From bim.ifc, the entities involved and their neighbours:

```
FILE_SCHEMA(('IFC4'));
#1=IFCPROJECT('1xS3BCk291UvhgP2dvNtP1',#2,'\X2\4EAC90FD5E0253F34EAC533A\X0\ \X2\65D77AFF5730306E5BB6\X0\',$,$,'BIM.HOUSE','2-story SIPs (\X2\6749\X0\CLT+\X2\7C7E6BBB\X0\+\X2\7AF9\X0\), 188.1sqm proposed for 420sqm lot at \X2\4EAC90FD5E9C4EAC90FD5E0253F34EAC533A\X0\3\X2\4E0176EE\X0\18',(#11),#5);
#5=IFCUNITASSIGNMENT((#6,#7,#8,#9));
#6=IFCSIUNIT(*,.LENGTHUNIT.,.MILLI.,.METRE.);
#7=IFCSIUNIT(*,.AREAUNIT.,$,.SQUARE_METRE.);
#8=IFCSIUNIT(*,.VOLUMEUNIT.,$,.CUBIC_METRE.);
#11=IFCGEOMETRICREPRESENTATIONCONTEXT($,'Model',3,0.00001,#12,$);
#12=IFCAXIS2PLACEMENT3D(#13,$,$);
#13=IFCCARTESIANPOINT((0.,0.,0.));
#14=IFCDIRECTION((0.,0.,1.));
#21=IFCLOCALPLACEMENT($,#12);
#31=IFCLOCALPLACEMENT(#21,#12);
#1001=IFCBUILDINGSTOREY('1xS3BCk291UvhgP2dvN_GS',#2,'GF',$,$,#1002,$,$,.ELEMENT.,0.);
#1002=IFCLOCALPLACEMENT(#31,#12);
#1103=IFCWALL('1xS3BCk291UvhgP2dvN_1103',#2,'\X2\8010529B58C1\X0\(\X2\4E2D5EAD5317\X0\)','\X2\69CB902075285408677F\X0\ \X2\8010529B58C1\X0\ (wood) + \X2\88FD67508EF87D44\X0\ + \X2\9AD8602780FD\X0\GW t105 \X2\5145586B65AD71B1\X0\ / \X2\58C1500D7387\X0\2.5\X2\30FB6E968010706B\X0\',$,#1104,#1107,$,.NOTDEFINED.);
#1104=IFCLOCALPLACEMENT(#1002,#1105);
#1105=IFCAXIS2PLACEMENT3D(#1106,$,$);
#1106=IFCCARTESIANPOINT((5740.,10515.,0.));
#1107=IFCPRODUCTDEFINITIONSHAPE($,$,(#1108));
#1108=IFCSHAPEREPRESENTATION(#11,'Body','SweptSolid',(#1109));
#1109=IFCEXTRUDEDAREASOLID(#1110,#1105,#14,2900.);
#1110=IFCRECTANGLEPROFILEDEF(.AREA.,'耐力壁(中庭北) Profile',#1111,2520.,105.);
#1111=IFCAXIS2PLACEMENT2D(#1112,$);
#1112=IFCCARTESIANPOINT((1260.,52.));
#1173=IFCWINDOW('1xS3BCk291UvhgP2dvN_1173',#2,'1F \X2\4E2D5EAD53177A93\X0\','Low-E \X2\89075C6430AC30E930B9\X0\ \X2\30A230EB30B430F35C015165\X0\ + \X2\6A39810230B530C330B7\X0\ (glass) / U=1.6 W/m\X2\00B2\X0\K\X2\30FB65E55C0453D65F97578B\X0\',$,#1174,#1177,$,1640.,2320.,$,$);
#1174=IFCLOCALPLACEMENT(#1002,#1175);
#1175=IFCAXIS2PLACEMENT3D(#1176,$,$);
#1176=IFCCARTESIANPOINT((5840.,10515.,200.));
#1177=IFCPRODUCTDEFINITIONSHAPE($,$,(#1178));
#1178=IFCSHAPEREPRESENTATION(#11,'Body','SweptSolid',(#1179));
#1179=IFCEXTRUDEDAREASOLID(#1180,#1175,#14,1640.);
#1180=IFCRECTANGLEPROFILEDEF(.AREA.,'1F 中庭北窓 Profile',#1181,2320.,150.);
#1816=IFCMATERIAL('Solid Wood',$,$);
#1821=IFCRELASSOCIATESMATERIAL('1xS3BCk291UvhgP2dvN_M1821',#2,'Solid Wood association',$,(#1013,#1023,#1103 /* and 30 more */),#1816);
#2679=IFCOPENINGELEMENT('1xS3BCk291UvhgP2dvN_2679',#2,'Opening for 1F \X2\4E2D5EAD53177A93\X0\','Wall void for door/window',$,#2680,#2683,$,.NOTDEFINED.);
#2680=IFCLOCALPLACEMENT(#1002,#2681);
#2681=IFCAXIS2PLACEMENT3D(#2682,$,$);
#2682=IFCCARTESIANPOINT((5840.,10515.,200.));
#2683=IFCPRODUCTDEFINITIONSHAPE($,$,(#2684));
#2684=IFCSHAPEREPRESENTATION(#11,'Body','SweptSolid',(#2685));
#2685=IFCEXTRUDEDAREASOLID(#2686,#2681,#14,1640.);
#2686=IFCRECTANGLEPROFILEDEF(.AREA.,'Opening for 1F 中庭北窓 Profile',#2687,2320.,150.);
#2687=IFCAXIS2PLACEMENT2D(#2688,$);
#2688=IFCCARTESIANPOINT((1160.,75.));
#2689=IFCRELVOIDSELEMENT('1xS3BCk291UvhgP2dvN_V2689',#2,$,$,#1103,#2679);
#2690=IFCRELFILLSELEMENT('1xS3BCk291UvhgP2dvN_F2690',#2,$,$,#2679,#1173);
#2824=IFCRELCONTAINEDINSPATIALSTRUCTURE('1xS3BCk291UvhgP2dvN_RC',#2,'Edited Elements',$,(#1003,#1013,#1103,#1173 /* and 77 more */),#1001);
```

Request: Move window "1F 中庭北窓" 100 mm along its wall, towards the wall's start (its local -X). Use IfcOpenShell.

```python
import ifcopenshell
import ifcopenshell.api.geometry
import ifcopenshell.util.placement
import ifcopenshell.util.unit

model = ifcopenshell.open("bim.ifc")
unit_scale = ifcopenshell.util.unit.calculate_unit_scale(model)

window = model.by_guid("1xS3BCk291UvhgP2dvN_1173")
opening = window.FillsVoids[0].RelatingOpeningElement
wall = opening.VoidsElements[0].RelatingBuildingElement

wall_matrix = ifcopenshell.util.placement.get_local_placement(wall.ObjectPlacement)
shift = wall_matrix[:3, 0] * -0.1 / unit_scale
before = ifcopenshell.util.placement.get_local_placement(window.ObjectPlacement)[:3, 3].copy()

# The window is not placed relative to its opening, so move both.
for product in (opening, window):
    matrix = ifcopenshell.util.placement.get_local_placement(product.ObjectPlacement)
    matrix[:3, 3] += shift
    ifcopenshell.api.geometry.edit_object_placement(model, product=product, matrix=matrix, is_si=False)

after = ifcopenshell.util.placement.get_local_placement(window.ObjectPlacement)[:3, 3]
print("window moved by", (after - before).round(3) + 0.0)

model.write("bim_rev.ifc")
```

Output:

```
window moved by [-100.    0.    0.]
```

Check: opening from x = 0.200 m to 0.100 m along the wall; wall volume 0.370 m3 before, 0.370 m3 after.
